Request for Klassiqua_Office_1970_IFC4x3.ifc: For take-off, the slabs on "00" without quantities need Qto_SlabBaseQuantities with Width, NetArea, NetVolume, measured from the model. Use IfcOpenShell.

First a look at what the model holds.

```python
import ifcopenshell
import ifcopenshell.util.element
import ifcopenshell.util.unit

model = ifcopenshell.open("Klassiqua_Office_1970_IFC4x3.ifc")
print(model.schema)
for unit_type in ("LENGTHUNIT", "AREAUNIT", "VOLUMEUNIT"):
    print(unit_type, ifcopenshell.util.unit.calculate_unit_scale(model, unit_type))
storey = next(s for s in model.by_type("IfcBuildingStorey") if s.Name == "00")
slabs = [e for e in ifcopenshell.util.element.get_decomposition(storey) if e.is_a("IfcSlab")]
for e in sorted(slabs, key=lambda e: e.id()):
    print(e.id(), e.is_a(), e.Name, list(ifcopenshell.util.element.get_psets(e, qtos_only=True)), sep=" | ")
```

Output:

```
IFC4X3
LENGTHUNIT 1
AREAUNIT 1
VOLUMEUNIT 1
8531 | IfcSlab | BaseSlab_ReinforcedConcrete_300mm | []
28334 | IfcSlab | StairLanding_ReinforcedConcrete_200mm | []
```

```python
import ifcopenshell
import ifcopenshell.api.pset
import ifcopenshell.geom
import ifcopenshell.util.element
import ifcopenshell.util.shape
import ifcopenshell.util.unit

model = ifcopenshell.open("Klassiqua_Office_1970_IFC4x3.ifc")
unit_scale = ifcopenshell.util.unit.calculate_unit_scale(model)
area_scale = ifcopenshell.util.unit.calculate_unit_scale(model, "AREAUNIT")
volume_scale = ifcopenshell.util.unit.calculate_unit_scale(model, "VOLUMEUNIT")
settings = ifcopenshell.geom.settings()

storey = next(s for s in model.by_type("IfcBuildingStorey") if s.Name == "00")
slabs = [e for e in ifcopenshell.util.element.get_decomposition(storey) if e.is_a("IfcSlab")]

for e in sorted(slabs, key=lambda e: e.id()):
    if ifcopenshell.util.element.get_psets(e, qtos_only=True, should_inherit=False):
        continue
    # Geometry comes back in metres, in the element's own axes.
    shape = ifcopenshell.geom.create_shape(settings, e)
    values = {
        "Width": ifcopenshell.util.shape.get_z(shape.geometry) / unit_scale,
        "NetArea": ifcopenshell.util.shape.get_footprint_area(shape.geometry) / area_scale,
        "NetVolume": ifcopenshell.util.shape.get_volume(shape.geometry) / volume_scale,
    }
    qto = ifcopenshell.api.pset.add_qto(model, product=e, name="Qto_SlabBaseQuantities")
    ifcopenshell.api.pset.edit_qto(model, qto=qto, properties=values)
    print(e.id(), {k: round(v, 3) for k, v in values.items()})

model.write("Klassiqua_Office_1970_IFC4x3_edited.ifc")
```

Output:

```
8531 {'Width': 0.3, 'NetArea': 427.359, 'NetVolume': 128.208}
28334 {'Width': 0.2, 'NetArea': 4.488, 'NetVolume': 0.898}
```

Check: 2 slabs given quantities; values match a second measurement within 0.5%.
